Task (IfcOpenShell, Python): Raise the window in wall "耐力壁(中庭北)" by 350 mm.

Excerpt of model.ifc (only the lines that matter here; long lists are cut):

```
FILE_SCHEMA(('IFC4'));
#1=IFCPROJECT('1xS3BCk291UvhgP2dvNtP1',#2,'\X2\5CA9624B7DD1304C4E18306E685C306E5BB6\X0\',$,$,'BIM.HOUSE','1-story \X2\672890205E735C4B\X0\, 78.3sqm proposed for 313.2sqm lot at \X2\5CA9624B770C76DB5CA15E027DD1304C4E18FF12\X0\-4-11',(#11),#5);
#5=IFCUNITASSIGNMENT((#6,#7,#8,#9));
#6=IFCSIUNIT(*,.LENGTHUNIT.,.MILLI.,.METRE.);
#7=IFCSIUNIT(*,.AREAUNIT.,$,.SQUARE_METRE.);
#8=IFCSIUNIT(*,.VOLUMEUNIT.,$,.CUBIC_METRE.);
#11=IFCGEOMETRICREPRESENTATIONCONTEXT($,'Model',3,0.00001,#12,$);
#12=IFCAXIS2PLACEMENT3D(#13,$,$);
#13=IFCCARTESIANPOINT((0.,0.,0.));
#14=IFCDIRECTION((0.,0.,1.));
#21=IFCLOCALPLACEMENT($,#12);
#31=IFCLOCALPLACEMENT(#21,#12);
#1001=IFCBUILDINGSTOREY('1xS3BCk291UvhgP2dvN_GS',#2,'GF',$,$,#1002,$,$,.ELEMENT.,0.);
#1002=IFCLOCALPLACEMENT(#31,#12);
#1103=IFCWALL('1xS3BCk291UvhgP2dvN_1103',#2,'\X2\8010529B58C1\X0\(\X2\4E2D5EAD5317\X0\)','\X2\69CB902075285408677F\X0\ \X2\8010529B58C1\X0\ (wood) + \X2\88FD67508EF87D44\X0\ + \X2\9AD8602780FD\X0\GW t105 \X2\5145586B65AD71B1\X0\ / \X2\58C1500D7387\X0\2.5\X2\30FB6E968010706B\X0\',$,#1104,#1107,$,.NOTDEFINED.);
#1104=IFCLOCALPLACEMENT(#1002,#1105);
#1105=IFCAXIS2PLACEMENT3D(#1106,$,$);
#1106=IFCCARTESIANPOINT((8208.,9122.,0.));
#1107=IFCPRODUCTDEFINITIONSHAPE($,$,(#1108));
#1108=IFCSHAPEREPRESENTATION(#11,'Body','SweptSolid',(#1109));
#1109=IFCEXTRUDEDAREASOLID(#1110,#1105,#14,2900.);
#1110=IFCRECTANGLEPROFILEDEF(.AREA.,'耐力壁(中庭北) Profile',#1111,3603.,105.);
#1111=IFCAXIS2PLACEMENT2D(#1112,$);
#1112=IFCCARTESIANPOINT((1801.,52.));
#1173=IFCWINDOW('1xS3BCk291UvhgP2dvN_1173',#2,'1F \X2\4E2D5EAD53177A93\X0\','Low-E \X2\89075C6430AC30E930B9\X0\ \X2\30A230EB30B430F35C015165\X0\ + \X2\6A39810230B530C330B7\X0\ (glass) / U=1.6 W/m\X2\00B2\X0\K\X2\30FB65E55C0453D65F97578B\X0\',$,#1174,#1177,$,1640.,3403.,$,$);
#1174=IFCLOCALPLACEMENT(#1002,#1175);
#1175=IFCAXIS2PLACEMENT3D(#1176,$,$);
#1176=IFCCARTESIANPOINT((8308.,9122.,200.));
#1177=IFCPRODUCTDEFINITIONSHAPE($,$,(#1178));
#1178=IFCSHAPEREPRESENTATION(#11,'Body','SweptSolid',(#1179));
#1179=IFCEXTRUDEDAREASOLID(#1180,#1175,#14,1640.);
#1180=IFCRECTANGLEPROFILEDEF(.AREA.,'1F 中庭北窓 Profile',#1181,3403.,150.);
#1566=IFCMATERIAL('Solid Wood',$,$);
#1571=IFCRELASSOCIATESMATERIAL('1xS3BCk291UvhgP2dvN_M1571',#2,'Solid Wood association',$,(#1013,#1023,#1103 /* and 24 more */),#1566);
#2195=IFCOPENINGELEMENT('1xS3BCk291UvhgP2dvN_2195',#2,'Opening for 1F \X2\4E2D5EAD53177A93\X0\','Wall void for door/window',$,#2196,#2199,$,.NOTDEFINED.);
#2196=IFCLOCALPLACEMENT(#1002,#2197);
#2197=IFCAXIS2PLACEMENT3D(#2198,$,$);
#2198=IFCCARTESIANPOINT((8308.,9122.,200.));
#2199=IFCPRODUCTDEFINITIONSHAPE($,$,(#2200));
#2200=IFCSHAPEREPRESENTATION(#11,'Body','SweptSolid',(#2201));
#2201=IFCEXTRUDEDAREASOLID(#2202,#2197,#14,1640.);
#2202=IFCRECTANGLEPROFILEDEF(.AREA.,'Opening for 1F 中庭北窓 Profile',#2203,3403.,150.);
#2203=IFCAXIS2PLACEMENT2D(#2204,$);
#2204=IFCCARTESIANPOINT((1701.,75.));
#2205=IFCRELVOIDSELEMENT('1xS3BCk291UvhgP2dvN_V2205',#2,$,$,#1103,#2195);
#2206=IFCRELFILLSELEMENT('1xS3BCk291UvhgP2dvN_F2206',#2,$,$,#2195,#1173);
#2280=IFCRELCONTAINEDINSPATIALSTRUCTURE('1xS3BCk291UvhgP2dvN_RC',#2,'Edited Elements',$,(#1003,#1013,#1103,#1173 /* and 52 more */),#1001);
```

```python
import numpy as np
import ifcopenshell
import ifcopenshell.api.geometry
import ifcopenshell.util.placement
import ifcopenshell.util.unit

model = ifcopenshell.open("model.ifc")
unit_scale = ifcopenshell.util.unit.calculate_unit_scale(model)

window = model.by_guid("1xS3BCk291UvhgP2dvN_1173")
opening = window.FillsVoids[0].RelatingOpeningElement
dz = 0.35 / unit_scale

shift = np.array([0.0, 0.0, dz])
# The window is not placed relative to its opening, so move both.
for product in (opening, window):
    matrix = ifcopenshell.util.placement.get_local_placement(product.ObjectPlacement)
    matrix[:3, 3] += shift
    ifcopenshell.api.geometry.edit_object_placement(model, product=product, matrix=matrix, is_si=False)

print(f"moved by {dz * unit_scale:+.3f} m")

model.write("model_rev.ifc")
```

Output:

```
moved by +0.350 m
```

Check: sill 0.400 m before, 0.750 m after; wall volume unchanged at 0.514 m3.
